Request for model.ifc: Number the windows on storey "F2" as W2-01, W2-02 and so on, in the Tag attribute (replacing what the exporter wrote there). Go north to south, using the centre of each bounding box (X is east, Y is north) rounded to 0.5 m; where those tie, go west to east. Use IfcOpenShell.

First a look at what the model holds.

```python
import ifcopenshell
import ifcopenshell.util.element
import ifcopenshell.util.placement

model = ifcopenshell.open("model.ifc")
print(model.schema)
storey = next(s for s in model.by_type("IfcBuildingStorey") if s.Name == "F2")
windows = [e for e in ifcopenshell.util.element.get_decomposition(storey) if e.is_a("IfcWindow")]
for e in sorted(windows, key=lambda e: e.id()):
    origin = ifcopenshell.util.placement.get_local_placement(e.ObjectPlacement)[:3, 3]
    print(e.id(), e.Tag, e.Name, origin.round(2) + 0.0, sep=" | ")
```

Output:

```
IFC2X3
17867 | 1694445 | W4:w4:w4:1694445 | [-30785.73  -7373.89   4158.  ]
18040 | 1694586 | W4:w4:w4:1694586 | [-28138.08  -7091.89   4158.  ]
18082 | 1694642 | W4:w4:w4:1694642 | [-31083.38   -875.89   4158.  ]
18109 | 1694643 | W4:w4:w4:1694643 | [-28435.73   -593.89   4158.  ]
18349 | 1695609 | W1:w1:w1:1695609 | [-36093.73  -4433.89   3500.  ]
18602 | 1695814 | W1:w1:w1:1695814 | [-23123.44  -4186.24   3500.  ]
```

```python
import ifcopenshell
import ifcopenshell.geom
import ifcopenshell.util.element
import ifcopenshell.util.shape

model = ifcopenshell.open("model.ifc")
settings = ifcopenshell.geom.settings()
settings.set("use-world-coords", True)


def centre(element):
    shape = ifcopenshell.geom.create_shape(settings, element)
    return ifcopenshell.util.shape.get_bbox_centroid(shape.geometry)


storey = next(s for s in model.by_type("IfcBuildingStorey") if s.Name == "F2")
windows = [e for e in ifcopenshell.util.element.get_decomposition(storey) if e.is_a("IfcWindow")]

# Insertion points can sit at a corner or the storey origin, so sort by the geometry (in metres).
centres = {e: centre(e) for e in windows}
windows.sort(key=lambda e: (-round(centres[e][1] / 0.5), centres[e][0]))

for i, e in enumerate(windows, start=1):
    number = f"W2-{i:02d}"
    e.Tag = number
    print(e.id(), number)

model.write("model_updated.ifc")
```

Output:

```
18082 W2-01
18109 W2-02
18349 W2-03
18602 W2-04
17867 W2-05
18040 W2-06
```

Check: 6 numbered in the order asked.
